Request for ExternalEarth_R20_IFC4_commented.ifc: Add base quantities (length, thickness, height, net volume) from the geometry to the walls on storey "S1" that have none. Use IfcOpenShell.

First a look at what the model holds.

```python
import ifcopenshell
import ifcopenshell.util.element
import ifcopenshell.util.unit

model = ifcopenshell.open("ExternalEarth_R20_IFC4_commented.ifc")
print(model.schema)
for unit_type in ("LENGTHUNIT", "AREAUNIT", "VOLUMEUNIT"):
    print(unit_type, ifcopenshell.util.unit.calculate_unit_scale(model, unit_type))
storey = next(s for s in model.by_type("IfcBuildingStorey") if s.Name == "S1")
walls = [e for e in ifcopenshell.util.element.get_decomposition(storey) if e.is_a("IfcWall")]
for e in sorted(walls, key=lambda e: e.id()):
    print(e.id(), e.is_a(), e.Name, list(ifcopenshell.util.element.get_psets(e, qtos_only=True)), sep=" | ")
```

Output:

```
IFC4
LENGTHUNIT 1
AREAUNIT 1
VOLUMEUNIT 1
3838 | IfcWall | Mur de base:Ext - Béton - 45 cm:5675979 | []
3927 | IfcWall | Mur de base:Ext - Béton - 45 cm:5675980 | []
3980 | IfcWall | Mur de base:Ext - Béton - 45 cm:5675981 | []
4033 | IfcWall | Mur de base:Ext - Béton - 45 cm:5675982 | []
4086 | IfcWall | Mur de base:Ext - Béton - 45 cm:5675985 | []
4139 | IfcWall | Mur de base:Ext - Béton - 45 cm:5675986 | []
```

```python
import ifcopenshell
import ifcopenshell.api.pset
import ifcopenshell.geom
import ifcopenshell.util.element
import ifcopenshell.util.shape
import ifcopenshell.util.unit

model = ifcopenshell.open("ExternalEarth_R20_IFC4_commented.ifc")
unit_scale = ifcopenshell.util.unit.calculate_unit_scale(model)
volume_scale = ifcopenshell.util.unit.calculate_unit_scale(model, "VOLUMEUNIT")
settings = ifcopenshell.geom.settings()

storey = next(s for s in model.by_type("IfcBuildingStorey") if s.Name == "S1")
walls = [e for e in ifcopenshell.util.element.get_decomposition(storey) if e.is_a("IfcWall")]

for e in sorted(walls, key=lambda e: e.id()):
    if ifcopenshell.util.element.get_psets(e, qtos_only=True, should_inherit=False):
        continue
    # Geometry comes back in metres, in the element's own axes.
    shape = ifcopenshell.geom.create_shape(settings, e)
    values = {
        "Length": ifcopenshell.util.shape.get_x(shape.geometry) / unit_scale,
        "Width": ifcopenshell.util.shape.get_y(shape.geometry) / unit_scale,
        "Height": ifcopenshell.util.shape.get_z(shape.geometry) / unit_scale,
        "NetVolume": ifcopenshell.util.shape.get_volume(shape.geometry) / volume_scale,
    }
    qto = ifcopenshell.api.pset.add_qto(model, product=e, name="Qto_WallBaseQuantities")
    ifcopenshell.api.pset.edit_qto(model, qto=qto, properties=values)
    print(e.id(), {k: round(v, 3) for k, v in values.items()})

model.write("ExternalEarth_R20_IFC4_commented_rev.ifc")
```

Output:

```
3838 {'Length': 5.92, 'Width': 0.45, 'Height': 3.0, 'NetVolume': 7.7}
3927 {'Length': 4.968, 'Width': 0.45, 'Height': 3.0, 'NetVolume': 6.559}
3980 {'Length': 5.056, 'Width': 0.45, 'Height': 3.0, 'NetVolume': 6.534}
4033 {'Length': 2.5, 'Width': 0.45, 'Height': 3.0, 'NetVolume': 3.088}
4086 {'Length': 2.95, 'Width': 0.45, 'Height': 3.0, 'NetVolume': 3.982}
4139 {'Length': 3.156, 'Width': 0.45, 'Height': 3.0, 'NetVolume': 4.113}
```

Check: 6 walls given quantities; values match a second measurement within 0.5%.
